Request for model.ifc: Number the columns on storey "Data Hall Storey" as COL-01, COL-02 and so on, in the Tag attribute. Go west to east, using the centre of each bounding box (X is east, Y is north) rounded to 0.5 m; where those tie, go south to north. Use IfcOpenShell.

First a look at what the model holds.

```python
import ifcopenshell
import ifcopenshell.util.element
import ifcopenshell.util.placement

model = ifcopenshell.open("model.ifc")
print(model.schema)
storey = next(s for s in model.by_type("IfcBuildingStorey") if s.Name == "Data Hall Storey")
columns = [e for e in ifcopenshell.util.element.get_decomposition(storey) if e.is_a("IfcColumn")]
for e in sorted(columns, key=lambda e: e.id()):
    origin = ifcopenshell.util.placement.get_local_placement(e.ObjectPlacement)[:3, 3]
    print(e.id(), e.Tag, e.Name, origin.round(2) + 0.0, sep=" | ")
```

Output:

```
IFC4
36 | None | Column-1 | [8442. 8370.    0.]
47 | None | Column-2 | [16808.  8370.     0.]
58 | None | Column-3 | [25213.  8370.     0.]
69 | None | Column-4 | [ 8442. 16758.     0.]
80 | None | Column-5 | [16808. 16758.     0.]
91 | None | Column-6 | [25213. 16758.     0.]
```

```python
import ifcopenshell
import ifcopenshell.geom
import ifcopenshell.util.element
import ifcopenshell.util.shape

model = ifcopenshell.open("model.ifc")
settings = ifcopenshell.geom.settings()
settings.set("use-world-coords", True)


def centre(element):
    shape = ifcopenshell.geom.create_shape(settings, element)
    return ifcopenshell.util.shape.get_bbox_centroid(shape.geometry)


storey = next(s for s in model.by_type("IfcBuildingStorey") if s.Name == "Data Hall Storey")
columns = [e for e in ifcopenshell.util.element.get_decomposition(storey) if e.is_a("IfcColumn")]

# Insertion points can sit at a corner or the storey origin, so sort by the geometry (in metres).
centres = {e: centre(e) for e in columns}
columns.sort(key=lambda e: (round(centres[e][0] / 0.5), centres[e][1]))

for i, e in enumerate(columns, start=1):
    number = f"COL-{i:02d}"
    e.Tag = number
    print(e.id(), number)

model.write("model_rev.ifc")
```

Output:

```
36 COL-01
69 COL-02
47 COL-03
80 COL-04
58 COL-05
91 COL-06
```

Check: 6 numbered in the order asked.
